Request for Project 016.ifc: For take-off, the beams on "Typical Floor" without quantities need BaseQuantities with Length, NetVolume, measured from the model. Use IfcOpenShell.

First a look at what the model holds.

```python
import ifcopenshell
import ifcopenshell.util.element
import ifcopenshell.util.unit

model = ifcopenshell.open("Project 016.ifc")
print(model.schema)
for unit_type in ("LENGTHUNIT", "AREAUNIT", "VOLUMEUNIT"):
    print(unit_type, ifcopenshell.util.unit.calculate_unit_scale(model, unit_type))
storey = next(s for s in model.by_type("IfcBuildingStorey") if s.Name == "Typical Floor")
beams = [e for e in ifcopenshell.util.element.get_decomposition(storey) if e.is_a("IfcBeam")]
for e in sorted(beams, key=lambda e: e.id()):
    print(e.id(), e.is_a(), e.Name, list(ifcopenshell.util.element.get_psets(e, qtos_only=True)), sep=" | ")
```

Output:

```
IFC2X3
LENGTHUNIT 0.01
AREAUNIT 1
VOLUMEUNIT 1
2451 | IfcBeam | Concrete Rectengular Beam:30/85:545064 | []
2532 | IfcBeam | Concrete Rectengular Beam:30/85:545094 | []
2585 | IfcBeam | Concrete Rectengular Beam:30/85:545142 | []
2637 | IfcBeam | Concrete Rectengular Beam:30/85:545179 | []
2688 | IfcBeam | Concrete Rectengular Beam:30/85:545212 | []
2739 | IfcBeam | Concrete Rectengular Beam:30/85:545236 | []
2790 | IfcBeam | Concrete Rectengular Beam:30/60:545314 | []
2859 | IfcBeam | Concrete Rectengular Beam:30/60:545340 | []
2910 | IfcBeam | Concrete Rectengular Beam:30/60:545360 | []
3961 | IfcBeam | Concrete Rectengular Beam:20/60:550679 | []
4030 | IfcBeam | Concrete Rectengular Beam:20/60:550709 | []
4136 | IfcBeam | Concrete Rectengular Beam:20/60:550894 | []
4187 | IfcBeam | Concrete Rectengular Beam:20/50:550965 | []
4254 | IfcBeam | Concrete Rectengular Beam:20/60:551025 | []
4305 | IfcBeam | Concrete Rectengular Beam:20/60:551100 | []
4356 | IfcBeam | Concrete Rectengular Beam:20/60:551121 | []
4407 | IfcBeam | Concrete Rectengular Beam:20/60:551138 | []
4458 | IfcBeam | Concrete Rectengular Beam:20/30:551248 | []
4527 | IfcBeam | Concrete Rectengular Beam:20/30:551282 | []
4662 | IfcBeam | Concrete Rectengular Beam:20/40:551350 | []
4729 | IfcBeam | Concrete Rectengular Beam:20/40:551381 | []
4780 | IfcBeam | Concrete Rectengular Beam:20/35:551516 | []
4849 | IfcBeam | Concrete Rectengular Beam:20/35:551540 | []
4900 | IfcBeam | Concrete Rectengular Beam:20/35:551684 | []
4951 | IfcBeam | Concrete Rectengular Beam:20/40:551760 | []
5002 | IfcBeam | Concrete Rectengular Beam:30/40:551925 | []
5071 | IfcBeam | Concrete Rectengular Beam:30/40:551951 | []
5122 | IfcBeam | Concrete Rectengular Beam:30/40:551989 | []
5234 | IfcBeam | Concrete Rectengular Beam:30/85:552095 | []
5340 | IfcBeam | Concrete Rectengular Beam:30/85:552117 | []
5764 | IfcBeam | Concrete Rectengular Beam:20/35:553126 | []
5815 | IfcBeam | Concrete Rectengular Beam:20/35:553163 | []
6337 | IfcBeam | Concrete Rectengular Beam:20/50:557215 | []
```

```python
import ifcopenshell
import ifcopenshell.api.pset
import ifcopenshell.geom
import ifcopenshell.util.element
import ifcopenshell.util.shape
import ifcopenshell.util.unit

model = ifcopenshell.open("Project 016.ifc")
unit_scale = ifcopenshell.util.unit.calculate_unit_scale(model)
volume_scale = ifcopenshell.util.unit.calculate_unit_scale(model, "VOLUMEUNIT")
settings = ifcopenshell.geom.settings()

storey = next(s for s in model.by_type("IfcBuildingStorey") if s.Name == "Typical Floor")
beams = [e for e in ifcopenshell.util.element.get_decomposition(storey) if e.is_a("IfcBeam")]

for e in sorted(beams, key=lambda e: e.id()):
    if ifcopenshell.util.element.get_psets(e, qtos_only=True, should_inherit=False):
        continue
    # Geometry comes back in metres, in the element's own axes.
    shape = ifcopenshell.geom.create_shape(settings, e)
    values = {
        "Length": ifcopenshell.util.shape.get_max_xyz(shape.geometry) / unit_scale,
        "NetVolume": ifcopenshell.util.shape.get_volume(shape.geometry) / volume_scale,
    }
    qto = ifcopenshell.api.pset.add_qto(model, product=e, name="BaseQuantities")
    ifcopenshell.api.pset.edit_qto(model, qto=qto, properties=values)
    print(e.id(), {k: round(v, 3) for k, v in values.items()})

model.write("Project 016_rev.ifc")
```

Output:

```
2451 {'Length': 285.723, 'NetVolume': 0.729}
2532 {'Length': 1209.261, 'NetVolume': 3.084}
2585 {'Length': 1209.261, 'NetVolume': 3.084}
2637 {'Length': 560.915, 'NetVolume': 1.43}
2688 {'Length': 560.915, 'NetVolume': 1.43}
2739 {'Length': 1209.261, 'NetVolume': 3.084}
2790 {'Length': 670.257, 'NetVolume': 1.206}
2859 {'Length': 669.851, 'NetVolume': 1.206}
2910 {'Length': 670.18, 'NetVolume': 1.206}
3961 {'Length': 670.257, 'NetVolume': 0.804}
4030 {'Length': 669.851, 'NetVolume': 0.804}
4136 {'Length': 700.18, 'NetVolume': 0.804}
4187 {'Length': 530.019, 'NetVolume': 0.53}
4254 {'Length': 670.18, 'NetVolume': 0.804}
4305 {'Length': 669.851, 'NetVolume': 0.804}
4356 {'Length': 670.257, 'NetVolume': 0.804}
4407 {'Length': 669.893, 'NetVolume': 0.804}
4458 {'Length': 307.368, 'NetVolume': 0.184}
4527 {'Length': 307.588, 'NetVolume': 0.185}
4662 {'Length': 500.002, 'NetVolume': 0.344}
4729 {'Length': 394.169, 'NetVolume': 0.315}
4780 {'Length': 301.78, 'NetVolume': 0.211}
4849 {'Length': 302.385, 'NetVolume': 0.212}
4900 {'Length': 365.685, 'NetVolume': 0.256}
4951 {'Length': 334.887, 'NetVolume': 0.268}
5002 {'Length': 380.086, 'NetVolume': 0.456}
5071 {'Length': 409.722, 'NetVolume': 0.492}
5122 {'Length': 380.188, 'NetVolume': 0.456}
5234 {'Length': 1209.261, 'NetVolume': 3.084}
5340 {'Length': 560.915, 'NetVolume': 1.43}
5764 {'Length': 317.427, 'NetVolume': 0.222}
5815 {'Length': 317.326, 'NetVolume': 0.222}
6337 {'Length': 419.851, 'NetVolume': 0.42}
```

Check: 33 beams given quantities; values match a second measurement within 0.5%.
